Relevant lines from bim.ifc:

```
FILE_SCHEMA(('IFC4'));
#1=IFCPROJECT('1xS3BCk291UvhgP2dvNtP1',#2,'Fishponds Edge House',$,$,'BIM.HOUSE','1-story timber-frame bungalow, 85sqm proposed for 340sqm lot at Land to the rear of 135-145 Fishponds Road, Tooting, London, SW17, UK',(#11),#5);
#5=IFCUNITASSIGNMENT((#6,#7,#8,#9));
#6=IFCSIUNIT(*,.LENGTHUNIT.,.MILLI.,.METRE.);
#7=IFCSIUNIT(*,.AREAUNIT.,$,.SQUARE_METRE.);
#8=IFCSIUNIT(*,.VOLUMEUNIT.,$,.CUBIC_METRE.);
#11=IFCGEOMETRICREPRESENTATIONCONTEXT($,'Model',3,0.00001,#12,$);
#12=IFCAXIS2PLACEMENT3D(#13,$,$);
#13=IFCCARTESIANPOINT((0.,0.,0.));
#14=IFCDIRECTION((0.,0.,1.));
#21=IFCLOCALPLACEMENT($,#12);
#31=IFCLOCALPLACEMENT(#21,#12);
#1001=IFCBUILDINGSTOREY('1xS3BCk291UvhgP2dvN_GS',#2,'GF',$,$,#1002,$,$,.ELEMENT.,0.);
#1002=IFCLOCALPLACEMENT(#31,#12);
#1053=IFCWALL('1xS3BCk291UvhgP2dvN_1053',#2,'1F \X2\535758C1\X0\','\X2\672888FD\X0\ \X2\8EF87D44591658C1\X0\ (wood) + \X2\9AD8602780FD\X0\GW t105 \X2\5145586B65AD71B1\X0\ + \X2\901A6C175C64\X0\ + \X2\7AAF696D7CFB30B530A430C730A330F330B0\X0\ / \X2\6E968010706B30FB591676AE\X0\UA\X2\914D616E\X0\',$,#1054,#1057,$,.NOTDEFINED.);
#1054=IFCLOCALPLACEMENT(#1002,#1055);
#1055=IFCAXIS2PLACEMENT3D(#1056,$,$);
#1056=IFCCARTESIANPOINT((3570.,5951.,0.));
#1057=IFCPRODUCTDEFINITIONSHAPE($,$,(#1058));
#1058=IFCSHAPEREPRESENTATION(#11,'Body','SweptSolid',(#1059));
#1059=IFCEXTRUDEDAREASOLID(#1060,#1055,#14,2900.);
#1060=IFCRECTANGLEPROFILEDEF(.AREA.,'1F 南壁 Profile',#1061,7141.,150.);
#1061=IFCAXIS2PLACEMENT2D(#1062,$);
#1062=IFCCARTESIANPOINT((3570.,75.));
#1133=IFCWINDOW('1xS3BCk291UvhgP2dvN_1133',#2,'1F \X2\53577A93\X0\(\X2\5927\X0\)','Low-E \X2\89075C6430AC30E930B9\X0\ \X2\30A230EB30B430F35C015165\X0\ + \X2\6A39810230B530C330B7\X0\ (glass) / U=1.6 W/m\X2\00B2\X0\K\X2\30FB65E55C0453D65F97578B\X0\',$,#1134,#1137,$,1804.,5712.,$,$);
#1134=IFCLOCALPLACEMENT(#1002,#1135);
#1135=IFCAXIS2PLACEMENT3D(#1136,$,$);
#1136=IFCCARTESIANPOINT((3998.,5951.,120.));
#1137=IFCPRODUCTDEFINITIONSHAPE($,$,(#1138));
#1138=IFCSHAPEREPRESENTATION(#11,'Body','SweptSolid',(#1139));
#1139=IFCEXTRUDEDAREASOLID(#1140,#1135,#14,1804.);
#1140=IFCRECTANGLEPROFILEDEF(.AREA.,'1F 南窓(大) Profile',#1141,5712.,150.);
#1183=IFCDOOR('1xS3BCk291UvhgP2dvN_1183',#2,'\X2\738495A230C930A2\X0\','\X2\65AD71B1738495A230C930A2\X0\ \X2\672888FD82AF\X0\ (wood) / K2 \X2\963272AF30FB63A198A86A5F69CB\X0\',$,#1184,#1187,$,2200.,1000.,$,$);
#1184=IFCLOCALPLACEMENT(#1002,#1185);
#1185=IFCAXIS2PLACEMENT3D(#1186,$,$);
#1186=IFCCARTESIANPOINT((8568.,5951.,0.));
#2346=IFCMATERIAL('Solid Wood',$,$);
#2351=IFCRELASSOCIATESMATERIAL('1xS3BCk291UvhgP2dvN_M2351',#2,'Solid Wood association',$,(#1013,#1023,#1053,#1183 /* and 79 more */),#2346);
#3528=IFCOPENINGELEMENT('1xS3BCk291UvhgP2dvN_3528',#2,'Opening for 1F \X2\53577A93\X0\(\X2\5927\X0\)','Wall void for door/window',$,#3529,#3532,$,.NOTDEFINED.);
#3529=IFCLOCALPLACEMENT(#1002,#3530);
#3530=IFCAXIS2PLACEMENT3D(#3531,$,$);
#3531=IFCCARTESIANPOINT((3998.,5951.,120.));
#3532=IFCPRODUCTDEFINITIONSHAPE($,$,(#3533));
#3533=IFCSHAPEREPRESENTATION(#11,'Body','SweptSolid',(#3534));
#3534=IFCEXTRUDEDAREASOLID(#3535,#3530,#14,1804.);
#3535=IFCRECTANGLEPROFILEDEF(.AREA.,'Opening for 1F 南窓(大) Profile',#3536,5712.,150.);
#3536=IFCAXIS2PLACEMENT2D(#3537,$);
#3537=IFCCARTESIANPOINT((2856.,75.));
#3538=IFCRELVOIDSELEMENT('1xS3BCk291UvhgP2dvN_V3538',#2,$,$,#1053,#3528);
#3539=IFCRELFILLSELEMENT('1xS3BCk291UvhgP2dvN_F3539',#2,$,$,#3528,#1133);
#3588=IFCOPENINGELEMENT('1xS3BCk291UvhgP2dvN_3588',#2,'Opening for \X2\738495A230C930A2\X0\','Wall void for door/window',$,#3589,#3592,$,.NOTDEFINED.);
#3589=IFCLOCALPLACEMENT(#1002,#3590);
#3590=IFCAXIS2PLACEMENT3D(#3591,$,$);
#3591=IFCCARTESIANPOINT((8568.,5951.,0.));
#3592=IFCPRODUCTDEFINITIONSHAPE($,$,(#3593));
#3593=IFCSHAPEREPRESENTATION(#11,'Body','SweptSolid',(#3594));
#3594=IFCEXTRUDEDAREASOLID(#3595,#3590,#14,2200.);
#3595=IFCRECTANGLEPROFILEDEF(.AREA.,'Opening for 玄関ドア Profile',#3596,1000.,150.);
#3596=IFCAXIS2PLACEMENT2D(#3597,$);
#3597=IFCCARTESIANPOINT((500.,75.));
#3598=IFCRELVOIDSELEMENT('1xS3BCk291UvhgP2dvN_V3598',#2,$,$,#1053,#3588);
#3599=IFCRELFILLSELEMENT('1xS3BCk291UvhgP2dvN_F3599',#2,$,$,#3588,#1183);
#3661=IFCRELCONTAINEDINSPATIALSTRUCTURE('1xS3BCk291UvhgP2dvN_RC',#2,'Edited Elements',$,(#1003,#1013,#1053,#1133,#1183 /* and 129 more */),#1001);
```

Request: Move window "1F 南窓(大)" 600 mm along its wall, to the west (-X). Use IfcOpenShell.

```python
import ifcopenshell
import ifcopenshell.api.geometry
import ifcopenshell.util.placement

model = ifcopenshell.open("bim.ifc")

window = model.by_id(1133)
opening = window.FillsVoids[0].RelatingOpeningElement
wall = opening.VoidsElements[0].RelatingBuildingElement

wall_matrix = ifcopenshell.util.placement.get_local_placement(wall.ObjectPlacement)
shift = wall_matrix[:3, 0] * -600.0
before = ifcopenshell.util.placement.get_local_placement(window.ObjectPlacement)[:3, 3].copy()

# The window is not placed relative to its opening, so move both.
for product in (opening, window):
    matrix = ifcopenshell.util.placement.get_local_placement(product.ObjectPlacement)
    matrix[:3, 3] += shift
    ifcopenshell.api.geometry.edit_object_placement(model, product=product, matrix=matrix, is_si=False)

after = ifcopenshell.util.placement.get_local_placement(window.ObjectPlacement)[:3, 3]
print("window moved by", (after - before).round(3) + 0.0)

model.write("bim-out.ifc")
```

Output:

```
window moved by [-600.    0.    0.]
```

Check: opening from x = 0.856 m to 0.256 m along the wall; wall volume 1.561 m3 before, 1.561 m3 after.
